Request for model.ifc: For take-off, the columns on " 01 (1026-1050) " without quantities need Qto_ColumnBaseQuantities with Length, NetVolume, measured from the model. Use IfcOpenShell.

First a look at what the model holds.

```python
import ifcopenshell
import ifcopenshell.util.element
import ifcopenshell.util.unit

model = ifcopenshell.open("model.ifc")
print(model.schema)
for unit_type in ("LENGTHUNIT", "AREAUNIT", "VOLUMEUNIT"):
    print(unit_type, ifcopenshell.util.unit.calculate_unit_scale(model, unit_type))
storey = next(s for s in model.by_type("IfcBuildingStorey") if s.Name == " 01 (1026-1050) ")
columns = [e for e in ifcopenshell.util.element.get_decomposition(storey) if e.is_a("IfcColumn")]
for e in sorted(columns, key=lambda e: e.id()):
    print(e.id(), e.is_a(), e.Name, list(ifcopenshell.util.element.get_psets(e, qtos_only=True)), sep=" | ")
```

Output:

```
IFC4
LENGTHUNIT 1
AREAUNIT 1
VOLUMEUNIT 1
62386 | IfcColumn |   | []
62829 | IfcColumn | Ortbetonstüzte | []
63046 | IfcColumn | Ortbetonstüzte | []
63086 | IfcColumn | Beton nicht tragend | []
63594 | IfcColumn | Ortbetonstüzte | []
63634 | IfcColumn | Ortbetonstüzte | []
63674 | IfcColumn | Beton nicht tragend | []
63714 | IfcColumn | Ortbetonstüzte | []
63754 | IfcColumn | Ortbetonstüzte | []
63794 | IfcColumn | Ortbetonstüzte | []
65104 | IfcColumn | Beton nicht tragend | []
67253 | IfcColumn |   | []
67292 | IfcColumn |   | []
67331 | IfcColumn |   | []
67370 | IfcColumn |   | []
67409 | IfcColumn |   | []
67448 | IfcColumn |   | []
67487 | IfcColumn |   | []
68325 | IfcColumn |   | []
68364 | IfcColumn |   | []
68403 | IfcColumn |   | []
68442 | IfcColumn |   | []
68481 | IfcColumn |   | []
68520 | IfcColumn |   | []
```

```python
import ifcopenshell
import ifcopenshell.api.pset
import ifcopenshell.geom
import ifcopenshell.util.element
import ifcopenshell.util.shape
import ifcopenshell.util.unit

model = ifcopenshell.open("model.ifc")
unit_scale = ifcopenshell.util.unit.calculate_unit_scale(model)
volume_scale = ifcopenshell.util.unit.calculate_unit_scale(model, "VOLUMEUNIT")
settings = ifcopenshell.geom.settings()

storey = next(s for s in model.by_type("IfcBuildingStorey") if s.Name == " 01 (1026-1050) ")
columns = [e for e in ifcopenshell.util.element.get_decomposition(storey) if e.is_a("IfcColumn")]

for e in sorted(columns, key=lambda e: e.id()):
    if ifcopenshell.util.element.get_psets(e, qtos_only=True, should_inherit=False):
        continue
    # Geometry comes back in metres, in the element's own axes.
    shape = ifcopenshell.geom.create_shape(settings, e)
    values = {
        "Length": ifcopenshell.util.shape.get_z(shape.geometry) / unit_scale,
        "NetVolume": ifcopenshell.util.shape.get_volume(shape.geometry) / volume_scale,
    }
    qto = ifcopenshell.api.pset.add_qto(model, product=e, name="Qto_ColumnBaseQuantities")
    ifcopenshell.api.pset.edit_qto(model, qto=qto, properties=values)
    print(e.id(), {k: round(v, 3) for k, v in values.items()})

model.write("model-out.ifc")
```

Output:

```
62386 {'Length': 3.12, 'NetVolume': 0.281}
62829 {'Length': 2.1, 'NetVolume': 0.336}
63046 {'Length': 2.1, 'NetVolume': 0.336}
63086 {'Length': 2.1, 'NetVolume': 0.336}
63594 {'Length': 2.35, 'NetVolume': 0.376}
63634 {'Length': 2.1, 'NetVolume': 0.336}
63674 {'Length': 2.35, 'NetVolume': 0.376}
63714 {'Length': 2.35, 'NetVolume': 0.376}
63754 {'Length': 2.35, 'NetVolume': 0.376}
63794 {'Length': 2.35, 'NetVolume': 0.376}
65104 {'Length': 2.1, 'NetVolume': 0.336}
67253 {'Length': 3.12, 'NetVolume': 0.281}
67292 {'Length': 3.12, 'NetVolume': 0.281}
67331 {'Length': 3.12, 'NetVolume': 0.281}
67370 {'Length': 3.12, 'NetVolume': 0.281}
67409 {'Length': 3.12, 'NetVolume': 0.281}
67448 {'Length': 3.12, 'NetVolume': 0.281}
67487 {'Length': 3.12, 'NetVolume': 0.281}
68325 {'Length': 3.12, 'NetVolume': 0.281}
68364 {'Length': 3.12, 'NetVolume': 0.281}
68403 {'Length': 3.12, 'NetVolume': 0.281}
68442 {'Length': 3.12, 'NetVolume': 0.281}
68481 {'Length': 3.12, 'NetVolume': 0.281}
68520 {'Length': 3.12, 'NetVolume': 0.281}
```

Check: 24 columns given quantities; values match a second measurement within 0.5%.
